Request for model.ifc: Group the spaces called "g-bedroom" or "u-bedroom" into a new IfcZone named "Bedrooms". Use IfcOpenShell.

First a look at what the model holds.

```python
import ifcopenshell

model = ifcopenshell.open("model.ifc")
print(model.schema)
seen = {}
for space in model.by_type("IfcSpace"):
    seen[space.LongName] = seen.get(space.LongName, 0) + 1
for name, count in sorted(seen.items(), key=str):
    print(count, "x", name)
print("zones:", [z.Name for z in model.by_type("IfcZone")][:20])
```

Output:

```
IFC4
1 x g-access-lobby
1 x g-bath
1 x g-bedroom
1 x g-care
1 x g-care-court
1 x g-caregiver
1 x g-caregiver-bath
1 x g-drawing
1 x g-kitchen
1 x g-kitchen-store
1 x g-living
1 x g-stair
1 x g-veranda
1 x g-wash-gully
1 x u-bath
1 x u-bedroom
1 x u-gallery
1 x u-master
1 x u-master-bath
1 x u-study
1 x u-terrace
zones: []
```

```python
import ifcopenshell
import ifcopenshell.api.group
import ifcopenshell.api.root

model = ifcopenshell.open("model.ifc")

names = {"g-bedroom", "u-bedroom"}
spaces = [s for s in model.by_type("IfcSpace") if s.LongName in names]

zone = ifcopenshell.api.root.create_entity(model, ifc_class="IfcZone", name="Bedrooms")
ifcopenshell.api.group.assign_group(model, products=spaces, group=zone)
print(len(spaces), "spaces in", zone.Name)

model.write("model_v2.ifc")
```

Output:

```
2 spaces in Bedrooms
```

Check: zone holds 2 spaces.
